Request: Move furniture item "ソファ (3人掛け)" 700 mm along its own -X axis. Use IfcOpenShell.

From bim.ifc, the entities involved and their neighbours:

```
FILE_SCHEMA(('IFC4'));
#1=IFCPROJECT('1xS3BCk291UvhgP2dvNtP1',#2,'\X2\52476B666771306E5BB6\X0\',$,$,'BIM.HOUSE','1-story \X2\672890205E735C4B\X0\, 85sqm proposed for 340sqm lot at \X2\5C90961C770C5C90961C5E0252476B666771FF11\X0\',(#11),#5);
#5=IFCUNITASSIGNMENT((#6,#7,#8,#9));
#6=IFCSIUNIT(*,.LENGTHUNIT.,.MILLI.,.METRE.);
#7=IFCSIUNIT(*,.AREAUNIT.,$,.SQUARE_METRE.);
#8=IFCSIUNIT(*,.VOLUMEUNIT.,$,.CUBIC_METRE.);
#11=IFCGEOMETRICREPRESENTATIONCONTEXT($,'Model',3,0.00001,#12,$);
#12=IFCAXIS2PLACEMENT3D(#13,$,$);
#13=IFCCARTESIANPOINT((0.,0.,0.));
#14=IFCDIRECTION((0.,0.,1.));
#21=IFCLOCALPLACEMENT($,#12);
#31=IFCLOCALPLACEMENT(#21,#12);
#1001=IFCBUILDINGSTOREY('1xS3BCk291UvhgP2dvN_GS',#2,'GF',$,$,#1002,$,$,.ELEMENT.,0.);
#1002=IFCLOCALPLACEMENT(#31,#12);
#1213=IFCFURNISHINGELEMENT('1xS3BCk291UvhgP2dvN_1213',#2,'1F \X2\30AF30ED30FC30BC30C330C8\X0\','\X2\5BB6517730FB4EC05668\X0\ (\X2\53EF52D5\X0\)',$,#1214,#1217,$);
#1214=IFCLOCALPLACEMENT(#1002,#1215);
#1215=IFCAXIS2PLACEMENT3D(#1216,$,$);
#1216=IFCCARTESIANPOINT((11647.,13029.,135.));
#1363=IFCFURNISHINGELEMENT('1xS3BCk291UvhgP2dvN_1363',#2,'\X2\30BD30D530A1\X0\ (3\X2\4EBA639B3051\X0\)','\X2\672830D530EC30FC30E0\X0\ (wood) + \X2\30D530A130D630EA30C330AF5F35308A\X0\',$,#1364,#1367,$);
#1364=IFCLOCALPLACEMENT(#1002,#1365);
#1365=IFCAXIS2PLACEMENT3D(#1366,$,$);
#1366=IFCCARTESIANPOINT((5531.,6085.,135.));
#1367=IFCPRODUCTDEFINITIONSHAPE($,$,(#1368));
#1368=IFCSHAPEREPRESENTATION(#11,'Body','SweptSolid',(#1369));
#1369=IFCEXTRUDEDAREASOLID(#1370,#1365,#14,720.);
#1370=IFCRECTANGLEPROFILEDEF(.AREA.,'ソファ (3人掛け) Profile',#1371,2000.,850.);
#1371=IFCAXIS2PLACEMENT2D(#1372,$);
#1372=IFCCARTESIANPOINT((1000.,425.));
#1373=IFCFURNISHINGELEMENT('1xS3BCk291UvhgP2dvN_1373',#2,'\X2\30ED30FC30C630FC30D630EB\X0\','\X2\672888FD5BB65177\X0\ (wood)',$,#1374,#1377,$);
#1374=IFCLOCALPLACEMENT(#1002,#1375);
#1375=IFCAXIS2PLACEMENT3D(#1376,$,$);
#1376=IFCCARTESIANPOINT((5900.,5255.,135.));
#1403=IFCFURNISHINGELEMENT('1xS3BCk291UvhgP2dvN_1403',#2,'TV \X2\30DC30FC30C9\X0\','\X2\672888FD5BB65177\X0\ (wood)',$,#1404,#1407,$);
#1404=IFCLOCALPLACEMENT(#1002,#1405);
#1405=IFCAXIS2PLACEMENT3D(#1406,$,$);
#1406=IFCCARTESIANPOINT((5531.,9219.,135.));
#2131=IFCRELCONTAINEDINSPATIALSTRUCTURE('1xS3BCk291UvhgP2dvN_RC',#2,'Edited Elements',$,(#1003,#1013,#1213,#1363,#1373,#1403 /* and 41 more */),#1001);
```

```python
import ifcopenshell
import ifcopenshell.api.geometry
import ifcopenshell.util.placement

model = ifcopenshell.open("bim.ifc")

item = model.by_id(1363)
matrix = ifcopenshell.util.placement.get_local_placement(item.ObjectPlacement)
matrix[:3, 3] -= matrix[:3, 0] * 700.0
ifcopenshell.api.geometry.edit_object_placement(model, product=item, matrix=matrix, is_si=False)

print(ifcopenshell.util.placement.get_local_placement(item.ObjectPlacement).round(3) + 0.0)

model.write("bim_updated.ifc")
```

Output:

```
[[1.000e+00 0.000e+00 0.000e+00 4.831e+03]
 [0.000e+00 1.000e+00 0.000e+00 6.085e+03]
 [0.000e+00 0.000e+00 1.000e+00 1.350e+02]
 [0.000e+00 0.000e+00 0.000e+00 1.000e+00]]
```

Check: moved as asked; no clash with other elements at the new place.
